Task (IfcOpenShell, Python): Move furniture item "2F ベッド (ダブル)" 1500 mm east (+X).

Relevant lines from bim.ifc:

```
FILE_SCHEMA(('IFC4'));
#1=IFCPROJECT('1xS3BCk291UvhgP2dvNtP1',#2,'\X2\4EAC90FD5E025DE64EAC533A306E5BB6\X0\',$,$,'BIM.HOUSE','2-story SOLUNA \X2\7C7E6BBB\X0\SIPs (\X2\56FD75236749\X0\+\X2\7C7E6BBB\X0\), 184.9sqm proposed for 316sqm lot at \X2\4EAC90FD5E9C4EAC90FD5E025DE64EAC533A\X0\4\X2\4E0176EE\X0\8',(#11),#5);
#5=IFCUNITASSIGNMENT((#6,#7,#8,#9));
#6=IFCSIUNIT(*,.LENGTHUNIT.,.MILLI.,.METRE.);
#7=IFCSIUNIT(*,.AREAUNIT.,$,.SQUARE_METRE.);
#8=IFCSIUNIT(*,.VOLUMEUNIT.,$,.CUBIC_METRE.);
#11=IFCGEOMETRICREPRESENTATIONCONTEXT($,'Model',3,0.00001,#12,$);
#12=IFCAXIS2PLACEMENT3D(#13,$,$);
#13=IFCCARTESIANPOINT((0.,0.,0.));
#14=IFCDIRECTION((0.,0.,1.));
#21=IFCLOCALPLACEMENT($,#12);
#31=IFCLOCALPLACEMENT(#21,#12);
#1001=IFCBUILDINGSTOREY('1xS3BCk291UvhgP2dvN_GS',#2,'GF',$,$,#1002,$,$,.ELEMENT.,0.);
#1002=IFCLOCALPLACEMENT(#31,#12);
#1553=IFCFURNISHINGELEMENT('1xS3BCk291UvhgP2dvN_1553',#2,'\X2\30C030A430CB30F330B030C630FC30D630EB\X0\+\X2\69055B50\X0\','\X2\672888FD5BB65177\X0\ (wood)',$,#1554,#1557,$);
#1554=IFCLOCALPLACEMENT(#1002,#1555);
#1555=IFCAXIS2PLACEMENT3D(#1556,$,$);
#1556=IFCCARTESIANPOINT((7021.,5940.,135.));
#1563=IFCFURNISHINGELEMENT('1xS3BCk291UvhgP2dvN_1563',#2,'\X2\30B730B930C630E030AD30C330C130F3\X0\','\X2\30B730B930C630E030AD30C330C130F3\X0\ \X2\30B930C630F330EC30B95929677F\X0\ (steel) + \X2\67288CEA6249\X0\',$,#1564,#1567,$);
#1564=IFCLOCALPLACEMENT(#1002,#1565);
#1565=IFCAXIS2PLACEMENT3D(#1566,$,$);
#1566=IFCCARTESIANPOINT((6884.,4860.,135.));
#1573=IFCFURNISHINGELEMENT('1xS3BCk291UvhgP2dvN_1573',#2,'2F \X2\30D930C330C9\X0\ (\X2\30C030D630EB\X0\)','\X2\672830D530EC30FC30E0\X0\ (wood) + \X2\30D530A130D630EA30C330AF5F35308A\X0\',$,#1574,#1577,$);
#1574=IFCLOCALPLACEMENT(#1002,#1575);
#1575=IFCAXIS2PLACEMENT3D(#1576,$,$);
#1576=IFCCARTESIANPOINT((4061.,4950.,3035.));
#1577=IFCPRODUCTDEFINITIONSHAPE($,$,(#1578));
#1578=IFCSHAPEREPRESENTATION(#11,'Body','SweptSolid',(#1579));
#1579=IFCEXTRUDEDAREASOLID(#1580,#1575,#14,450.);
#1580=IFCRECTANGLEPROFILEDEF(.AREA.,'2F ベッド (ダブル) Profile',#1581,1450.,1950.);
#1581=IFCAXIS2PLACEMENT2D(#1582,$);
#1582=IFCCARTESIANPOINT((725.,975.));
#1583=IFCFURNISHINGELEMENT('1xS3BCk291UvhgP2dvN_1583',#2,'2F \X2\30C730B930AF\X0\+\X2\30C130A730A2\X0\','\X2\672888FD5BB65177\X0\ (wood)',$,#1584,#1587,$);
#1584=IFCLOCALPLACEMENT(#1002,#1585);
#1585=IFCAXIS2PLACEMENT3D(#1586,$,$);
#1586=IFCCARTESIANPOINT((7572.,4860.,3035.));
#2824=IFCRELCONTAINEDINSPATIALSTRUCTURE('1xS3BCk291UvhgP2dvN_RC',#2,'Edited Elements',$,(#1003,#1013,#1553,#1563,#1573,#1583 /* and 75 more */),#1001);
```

```python
import ifcopenshell
import ifcopenshell.api.geometry
import ifcopenshell.util.placement

model = ifcopenshell.open("bim.ifc")

item = model.by_guid("1xS3BCk291UvhgP2dvN_1573")
matrix = ifcopenshell.util.placement.get_local_placement(item.ObjectPlacement)
matrix[0, 3] += 1500.0
ifcopenshell.api.geometry.edit_object_placement(model, product=item, matrix=matrix, is_si=False)

print(ifcopenshell.util.placement.get_local_placement(item.ObjectPlacement).round(3) + 0.0)

model.write("bim_v2.ifc")
```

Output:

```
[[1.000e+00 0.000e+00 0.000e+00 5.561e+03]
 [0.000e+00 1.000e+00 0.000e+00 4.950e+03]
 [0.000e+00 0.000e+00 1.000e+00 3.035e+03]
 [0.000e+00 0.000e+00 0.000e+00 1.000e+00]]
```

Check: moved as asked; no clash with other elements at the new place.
